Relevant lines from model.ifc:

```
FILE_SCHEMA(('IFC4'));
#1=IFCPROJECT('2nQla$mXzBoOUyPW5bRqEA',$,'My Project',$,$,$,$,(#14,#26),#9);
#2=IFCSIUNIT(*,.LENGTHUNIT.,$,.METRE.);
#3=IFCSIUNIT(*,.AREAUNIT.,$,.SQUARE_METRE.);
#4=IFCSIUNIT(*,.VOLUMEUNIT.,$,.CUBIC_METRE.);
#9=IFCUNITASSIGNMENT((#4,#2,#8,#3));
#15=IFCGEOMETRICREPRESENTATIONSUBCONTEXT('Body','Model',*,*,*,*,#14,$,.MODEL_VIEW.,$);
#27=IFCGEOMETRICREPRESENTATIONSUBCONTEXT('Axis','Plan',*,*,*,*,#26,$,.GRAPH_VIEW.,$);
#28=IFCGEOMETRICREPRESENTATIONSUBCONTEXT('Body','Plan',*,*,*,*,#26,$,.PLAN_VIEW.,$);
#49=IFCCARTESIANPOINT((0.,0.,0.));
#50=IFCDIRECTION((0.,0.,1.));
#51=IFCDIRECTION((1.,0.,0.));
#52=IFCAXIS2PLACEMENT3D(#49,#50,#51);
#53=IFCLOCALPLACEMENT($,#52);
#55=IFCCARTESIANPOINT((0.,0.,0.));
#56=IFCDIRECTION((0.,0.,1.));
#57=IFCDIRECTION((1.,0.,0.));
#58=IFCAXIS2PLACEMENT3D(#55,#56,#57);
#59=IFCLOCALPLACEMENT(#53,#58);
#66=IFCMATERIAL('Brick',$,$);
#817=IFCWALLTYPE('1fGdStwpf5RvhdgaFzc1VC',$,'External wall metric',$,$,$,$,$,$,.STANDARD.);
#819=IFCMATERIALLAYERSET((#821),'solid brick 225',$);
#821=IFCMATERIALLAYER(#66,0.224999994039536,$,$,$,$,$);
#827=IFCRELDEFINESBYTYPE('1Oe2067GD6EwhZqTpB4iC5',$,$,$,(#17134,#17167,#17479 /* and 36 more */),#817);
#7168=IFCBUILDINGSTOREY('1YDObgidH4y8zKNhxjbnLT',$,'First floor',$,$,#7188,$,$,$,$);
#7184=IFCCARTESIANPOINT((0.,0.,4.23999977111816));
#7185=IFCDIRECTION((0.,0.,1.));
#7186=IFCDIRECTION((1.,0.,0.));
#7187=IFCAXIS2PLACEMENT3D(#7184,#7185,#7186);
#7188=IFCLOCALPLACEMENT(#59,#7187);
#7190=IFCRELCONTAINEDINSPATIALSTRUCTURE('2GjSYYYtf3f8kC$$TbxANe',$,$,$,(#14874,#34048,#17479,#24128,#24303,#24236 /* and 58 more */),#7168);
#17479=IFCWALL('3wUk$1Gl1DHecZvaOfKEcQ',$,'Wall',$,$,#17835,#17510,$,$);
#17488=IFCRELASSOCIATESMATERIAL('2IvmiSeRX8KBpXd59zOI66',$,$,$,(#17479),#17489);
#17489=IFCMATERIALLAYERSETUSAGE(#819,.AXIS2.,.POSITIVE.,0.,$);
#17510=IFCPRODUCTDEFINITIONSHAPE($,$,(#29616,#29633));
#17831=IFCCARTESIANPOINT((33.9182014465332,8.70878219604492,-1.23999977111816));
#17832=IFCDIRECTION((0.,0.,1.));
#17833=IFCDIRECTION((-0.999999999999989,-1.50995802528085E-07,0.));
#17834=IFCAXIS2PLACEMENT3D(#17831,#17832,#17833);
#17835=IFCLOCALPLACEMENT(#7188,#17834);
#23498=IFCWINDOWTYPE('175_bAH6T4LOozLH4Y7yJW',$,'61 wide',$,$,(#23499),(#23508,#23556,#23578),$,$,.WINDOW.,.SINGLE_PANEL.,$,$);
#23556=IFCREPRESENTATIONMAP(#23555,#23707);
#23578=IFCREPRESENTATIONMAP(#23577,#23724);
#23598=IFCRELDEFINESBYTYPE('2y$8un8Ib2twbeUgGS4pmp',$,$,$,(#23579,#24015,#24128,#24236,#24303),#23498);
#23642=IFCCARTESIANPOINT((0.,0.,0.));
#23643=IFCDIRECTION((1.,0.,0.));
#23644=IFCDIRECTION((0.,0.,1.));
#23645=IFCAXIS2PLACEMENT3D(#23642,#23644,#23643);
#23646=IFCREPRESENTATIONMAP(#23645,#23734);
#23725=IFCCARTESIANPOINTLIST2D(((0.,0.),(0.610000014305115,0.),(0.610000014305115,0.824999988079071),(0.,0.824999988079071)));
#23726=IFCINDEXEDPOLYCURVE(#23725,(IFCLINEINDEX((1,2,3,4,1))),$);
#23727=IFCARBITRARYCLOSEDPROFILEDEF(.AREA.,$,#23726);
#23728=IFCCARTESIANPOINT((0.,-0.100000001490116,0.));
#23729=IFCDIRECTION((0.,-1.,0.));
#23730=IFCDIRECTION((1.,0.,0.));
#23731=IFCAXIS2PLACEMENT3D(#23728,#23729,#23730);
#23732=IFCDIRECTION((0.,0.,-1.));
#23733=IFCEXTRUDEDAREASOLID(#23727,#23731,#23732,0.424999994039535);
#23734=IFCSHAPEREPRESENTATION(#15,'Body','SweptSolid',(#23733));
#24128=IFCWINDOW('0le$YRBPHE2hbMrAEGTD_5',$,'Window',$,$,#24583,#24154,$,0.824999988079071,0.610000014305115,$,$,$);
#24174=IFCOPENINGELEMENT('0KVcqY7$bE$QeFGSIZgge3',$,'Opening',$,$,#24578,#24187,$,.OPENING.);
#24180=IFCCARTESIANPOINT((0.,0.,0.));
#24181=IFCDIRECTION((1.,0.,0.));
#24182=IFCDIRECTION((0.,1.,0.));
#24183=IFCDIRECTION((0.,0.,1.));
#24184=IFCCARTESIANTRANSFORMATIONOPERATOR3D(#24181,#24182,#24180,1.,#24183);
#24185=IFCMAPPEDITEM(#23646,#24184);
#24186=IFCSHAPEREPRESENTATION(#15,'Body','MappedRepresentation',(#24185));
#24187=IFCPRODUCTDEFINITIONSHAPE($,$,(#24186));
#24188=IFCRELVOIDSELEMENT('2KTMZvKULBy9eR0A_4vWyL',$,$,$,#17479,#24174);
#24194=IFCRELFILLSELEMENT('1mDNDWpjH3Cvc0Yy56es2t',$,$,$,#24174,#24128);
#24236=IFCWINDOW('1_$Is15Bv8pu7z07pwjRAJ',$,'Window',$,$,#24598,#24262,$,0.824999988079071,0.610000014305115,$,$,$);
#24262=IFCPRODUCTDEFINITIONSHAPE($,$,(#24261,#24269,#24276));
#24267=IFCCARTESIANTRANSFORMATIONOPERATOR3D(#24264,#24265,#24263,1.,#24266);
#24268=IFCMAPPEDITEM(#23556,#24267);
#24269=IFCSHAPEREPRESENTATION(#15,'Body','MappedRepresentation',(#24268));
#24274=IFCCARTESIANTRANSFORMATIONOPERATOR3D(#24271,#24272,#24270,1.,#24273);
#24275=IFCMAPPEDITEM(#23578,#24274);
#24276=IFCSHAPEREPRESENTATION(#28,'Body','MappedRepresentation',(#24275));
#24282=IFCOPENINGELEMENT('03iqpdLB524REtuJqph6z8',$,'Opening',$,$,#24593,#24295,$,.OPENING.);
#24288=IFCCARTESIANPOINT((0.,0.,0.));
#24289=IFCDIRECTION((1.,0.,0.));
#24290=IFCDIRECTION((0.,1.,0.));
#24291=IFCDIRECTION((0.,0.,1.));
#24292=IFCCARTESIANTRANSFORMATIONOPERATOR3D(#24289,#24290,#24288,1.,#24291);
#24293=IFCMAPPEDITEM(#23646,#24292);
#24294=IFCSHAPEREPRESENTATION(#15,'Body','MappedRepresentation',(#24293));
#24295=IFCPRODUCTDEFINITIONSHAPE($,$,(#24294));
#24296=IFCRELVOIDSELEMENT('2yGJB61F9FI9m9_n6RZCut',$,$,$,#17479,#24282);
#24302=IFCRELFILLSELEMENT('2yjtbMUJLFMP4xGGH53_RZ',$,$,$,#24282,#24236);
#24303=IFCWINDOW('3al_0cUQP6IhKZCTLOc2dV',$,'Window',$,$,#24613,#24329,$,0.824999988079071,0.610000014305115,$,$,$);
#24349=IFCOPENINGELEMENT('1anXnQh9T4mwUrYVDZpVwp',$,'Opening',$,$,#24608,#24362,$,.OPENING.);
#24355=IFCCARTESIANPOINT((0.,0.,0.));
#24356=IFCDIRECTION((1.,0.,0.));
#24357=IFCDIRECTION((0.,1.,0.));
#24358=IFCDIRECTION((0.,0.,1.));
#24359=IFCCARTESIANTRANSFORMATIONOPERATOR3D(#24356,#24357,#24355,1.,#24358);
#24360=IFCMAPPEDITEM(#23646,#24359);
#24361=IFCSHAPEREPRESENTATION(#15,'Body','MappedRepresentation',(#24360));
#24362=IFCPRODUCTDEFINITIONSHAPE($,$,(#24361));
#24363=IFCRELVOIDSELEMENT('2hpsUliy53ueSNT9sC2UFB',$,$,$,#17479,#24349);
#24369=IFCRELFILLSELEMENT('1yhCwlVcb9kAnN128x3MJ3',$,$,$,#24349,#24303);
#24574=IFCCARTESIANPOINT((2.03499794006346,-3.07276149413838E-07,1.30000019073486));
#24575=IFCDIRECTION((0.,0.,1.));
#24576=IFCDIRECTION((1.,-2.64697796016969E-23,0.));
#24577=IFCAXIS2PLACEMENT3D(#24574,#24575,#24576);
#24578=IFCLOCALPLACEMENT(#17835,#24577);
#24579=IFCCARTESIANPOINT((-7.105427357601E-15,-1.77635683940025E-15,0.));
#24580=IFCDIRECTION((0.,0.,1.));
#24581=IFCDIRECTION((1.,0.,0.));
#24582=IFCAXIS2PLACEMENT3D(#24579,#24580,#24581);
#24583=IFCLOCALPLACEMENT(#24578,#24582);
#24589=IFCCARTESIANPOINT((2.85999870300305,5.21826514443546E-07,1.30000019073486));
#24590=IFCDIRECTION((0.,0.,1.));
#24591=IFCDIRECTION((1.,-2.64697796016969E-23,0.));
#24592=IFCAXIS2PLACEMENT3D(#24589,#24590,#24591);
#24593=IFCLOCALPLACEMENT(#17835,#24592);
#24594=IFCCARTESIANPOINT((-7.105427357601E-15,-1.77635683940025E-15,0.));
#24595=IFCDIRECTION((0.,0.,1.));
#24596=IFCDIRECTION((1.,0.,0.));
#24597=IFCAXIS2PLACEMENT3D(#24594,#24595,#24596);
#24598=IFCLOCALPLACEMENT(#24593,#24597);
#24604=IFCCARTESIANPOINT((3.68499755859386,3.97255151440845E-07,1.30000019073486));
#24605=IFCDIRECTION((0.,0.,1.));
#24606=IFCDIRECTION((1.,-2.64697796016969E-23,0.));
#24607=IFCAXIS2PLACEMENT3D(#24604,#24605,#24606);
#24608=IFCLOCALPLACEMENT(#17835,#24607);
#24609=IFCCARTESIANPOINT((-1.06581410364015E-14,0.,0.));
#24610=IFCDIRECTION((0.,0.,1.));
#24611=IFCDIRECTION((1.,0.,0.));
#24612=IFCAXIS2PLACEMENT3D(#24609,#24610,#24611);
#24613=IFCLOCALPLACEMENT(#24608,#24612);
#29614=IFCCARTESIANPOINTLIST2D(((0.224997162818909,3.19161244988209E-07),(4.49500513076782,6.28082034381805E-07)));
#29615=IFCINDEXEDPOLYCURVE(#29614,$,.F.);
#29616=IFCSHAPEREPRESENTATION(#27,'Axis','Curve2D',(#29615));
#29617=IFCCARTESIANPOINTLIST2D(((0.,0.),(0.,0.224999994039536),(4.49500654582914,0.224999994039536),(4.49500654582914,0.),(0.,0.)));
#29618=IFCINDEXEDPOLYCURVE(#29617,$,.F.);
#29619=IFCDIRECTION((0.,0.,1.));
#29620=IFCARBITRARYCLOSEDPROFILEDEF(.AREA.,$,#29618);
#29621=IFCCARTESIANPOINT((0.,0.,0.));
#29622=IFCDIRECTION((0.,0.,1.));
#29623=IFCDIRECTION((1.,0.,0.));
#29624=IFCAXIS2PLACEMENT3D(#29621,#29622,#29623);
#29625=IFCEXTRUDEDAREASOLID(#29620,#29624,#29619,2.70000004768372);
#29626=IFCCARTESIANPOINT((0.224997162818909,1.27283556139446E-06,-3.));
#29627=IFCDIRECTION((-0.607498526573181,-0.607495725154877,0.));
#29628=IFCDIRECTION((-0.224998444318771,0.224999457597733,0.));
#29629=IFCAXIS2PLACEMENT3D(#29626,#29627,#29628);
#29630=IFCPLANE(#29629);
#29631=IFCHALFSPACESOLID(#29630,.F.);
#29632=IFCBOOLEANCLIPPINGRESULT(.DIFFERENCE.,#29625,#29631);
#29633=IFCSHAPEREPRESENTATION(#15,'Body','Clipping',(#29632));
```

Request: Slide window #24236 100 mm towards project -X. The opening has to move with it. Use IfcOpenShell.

```python
import ifcopenshell
import ifcopenshell.api.geometry
import ifcopenshell.util.placement

model = ifcopenshell.open("model.ifc")

window = model.by_guid("1_$Is15Bv8pu7z07pwjRAJ")
opening = window.FillsVoids[0].RelatingOpeningElement
wall = opening.VoidsElements[0].RelatingBuildingElement

wall_matrix = ifcopenshell.util.placement.get_local_placement(wall.ObjectPlacement)
shift = wall_matrix[:3, 0] * 0.1
before = ifcopenshell.util.placement.get_local_placement(window.ObjectPlacement)[:3, 3].copy()

# The window is placed relative to its opening, so it follows when the opening moves.
matrix = ifcopenshell.util.placement.get_local_placement(opening.ObjectPlacement)
matrix[:3, 3] += shift
ifcopenshell.api.geometry.edit_object_placement(
    model, product=opening, matrix=matrix, is_si=False, should_transform_children=True
)

after = ifcopenshell.util.placement.get_local_placement(window.ObjectPlacement)[:3, 3]
print("window moved by", (after - before).round(3) + 0.0)

model.write("model_edited.ifc")
```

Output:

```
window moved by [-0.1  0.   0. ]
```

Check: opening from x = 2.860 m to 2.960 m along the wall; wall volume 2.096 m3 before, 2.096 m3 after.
